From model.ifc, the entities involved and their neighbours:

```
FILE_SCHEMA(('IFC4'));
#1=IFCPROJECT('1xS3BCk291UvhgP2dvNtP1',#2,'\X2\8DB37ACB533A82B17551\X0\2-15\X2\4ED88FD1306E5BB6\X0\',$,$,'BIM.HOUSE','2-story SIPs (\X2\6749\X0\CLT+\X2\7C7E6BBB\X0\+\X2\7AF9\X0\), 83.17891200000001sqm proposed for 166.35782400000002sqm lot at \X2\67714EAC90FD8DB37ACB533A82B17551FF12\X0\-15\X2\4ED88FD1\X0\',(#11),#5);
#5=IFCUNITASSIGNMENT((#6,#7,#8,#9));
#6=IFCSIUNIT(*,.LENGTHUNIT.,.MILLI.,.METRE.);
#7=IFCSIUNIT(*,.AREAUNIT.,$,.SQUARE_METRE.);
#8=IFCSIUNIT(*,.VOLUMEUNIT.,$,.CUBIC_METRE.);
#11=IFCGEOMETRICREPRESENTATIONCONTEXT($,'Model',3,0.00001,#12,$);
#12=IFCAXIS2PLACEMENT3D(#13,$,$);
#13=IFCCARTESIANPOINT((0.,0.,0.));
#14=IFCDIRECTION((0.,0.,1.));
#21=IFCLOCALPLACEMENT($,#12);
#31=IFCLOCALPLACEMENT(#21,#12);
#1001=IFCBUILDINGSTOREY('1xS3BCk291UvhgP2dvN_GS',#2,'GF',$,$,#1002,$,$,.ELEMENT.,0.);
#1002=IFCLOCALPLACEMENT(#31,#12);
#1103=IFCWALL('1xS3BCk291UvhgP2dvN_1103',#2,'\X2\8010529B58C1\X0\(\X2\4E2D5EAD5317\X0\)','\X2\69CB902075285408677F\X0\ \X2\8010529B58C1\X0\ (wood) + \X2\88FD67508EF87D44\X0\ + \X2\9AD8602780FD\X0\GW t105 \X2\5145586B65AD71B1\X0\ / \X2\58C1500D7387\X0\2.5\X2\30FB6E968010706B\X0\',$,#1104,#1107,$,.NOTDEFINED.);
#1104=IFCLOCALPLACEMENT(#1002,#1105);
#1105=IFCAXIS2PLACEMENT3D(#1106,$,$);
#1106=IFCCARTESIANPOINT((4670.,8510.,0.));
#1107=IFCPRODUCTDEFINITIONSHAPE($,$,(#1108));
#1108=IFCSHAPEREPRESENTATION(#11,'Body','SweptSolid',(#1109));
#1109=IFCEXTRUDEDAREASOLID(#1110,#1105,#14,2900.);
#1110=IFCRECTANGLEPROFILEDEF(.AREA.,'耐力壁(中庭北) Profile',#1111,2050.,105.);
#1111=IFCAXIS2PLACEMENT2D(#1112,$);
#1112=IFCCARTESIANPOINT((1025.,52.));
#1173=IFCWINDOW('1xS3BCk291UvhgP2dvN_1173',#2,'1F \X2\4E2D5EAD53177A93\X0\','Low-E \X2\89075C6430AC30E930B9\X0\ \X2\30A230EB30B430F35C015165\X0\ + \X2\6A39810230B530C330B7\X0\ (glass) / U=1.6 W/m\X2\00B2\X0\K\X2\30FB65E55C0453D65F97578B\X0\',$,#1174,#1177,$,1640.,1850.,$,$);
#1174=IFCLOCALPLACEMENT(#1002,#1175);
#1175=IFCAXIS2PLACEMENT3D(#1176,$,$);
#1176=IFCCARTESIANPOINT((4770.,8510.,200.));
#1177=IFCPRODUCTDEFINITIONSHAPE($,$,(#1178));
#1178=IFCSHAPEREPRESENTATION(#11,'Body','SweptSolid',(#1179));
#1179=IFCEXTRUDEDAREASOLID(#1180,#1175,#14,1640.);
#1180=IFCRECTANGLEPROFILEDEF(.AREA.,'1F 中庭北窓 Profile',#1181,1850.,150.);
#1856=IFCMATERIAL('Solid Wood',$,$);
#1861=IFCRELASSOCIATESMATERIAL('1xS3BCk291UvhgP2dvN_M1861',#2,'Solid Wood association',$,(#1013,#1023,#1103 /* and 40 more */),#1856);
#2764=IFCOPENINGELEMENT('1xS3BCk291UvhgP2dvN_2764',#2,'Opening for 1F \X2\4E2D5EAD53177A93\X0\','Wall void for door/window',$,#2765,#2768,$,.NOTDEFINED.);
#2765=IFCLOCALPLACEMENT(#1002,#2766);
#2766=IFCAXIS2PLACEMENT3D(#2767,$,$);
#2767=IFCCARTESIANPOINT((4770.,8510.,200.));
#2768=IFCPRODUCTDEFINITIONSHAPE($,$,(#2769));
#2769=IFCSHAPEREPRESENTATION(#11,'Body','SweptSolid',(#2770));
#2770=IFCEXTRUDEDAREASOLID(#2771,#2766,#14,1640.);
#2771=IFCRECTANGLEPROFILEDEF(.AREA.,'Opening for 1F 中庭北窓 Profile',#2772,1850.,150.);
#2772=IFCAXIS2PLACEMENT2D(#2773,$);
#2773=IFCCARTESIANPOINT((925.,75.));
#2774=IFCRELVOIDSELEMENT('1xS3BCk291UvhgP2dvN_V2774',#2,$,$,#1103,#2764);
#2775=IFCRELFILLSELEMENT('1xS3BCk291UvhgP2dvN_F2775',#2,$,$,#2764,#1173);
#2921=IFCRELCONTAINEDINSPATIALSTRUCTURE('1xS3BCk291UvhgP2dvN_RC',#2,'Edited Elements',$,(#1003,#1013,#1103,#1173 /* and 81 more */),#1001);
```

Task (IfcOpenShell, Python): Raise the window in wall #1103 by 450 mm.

```python
import numpy as np
import ifcopenshell
import ifcopenshell.api.geometry
import ifcopenshell.util.placement
import ifcopenshell.util.unit

model = ifcopenshell.open("model.ifc")
unit_scale = ifcopenshell.util.unit.calculate_unit_scale(model)

window = model.by_guid("1xS3BCk291UvhgP2dvN_1173")
opening = window.FillsVoids[0].RelatingOpeningElement
dz = 450.0

shift = np.array([0.0, 0.0, dz])
# The window is not placed relative to its opening, so move both.
for product in (opening, window):
    matrix = ifcopenshell.util.placement.get_local_placement(product.ObjectPlacement)
    matrix[:3, 3] += shift
    ifcopenshell.api.geometry.edit_object_placement(model, product=product, matrix=matrix, is_si=False)

print(f"moved by {dz * unit_scale:+.3f} m")

model.write("model_updated.ifc")
```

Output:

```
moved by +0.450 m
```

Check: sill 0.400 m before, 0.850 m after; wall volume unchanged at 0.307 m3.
